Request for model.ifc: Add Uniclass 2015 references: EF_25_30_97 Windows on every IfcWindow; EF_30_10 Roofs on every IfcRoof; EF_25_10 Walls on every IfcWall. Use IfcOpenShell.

First a look at what the model holds.

```python
import ifcopenshell

model = ifcopenshell.open("model.ifc")
print(model.schema)
print("classifications:", [c.Name for c in model.by_type("IfcClassification")])
for ifc_class in ("IfcDoor", "IfcRoof", "IfcStair", "IfcWall", "IfcWindow"):
    print(ifc_class, len(model.by_type(ifc_class)))
```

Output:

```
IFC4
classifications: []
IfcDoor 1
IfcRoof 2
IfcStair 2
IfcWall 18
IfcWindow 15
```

```python
import ifcopenshell
import ifcopenshell.api.classification

model = ifcopenshell.open("model.ifc")

system = ifcopenshell.api.classification.add_classification(model, classification="Uniclass 2015")

codes = {
    "IfcWindow": ("EF_25_30_97", "Windows"),
    "IfcRoof": ("EF_30_10", "Roofs"),
    "IfcWall": ("EF_25_10", "Walls"),
}
for ifc_class, (code, name) in codes.items():
    products = model.by_type(ifc_class)
    ifcopenshell.api.classification.add_reference(
        model, products=products, classification=system, identification=code, name=name
    )
    print(code, len(products))

model.write("model_v2.ifc")
```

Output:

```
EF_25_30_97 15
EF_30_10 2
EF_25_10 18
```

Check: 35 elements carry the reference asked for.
